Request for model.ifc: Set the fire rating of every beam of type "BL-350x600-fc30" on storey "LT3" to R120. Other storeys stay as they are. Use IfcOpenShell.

First a look at what the model holds.

```python
import ifcopenshell
import ifcopenshell.util.element

model = ifcopenshell.open("model.ifc")
print(model.schema)
storey = next(s for s in model.by_type("IfcBuildingStorey") if s.Name == "LT3")
beams = [e for e in ifcopenshell.util.element.get_decomposition(storey) if e.is_a("IfcBeam")]
seen = {}
for e in beams:
    element_type = ifcopenshell.util.element.get_type(e)
    key = (element_type.Name if element_type != e and element_type else None, ifcopenshell.util.element.get_pset(e, "Pset_BeamCommon", "FireRating"))
    seen[key] = seen.get(key, 0) + 1
for (name, value), count in sorted(seen.items(), key=str):
    print(count, "x", name, "|", value)
```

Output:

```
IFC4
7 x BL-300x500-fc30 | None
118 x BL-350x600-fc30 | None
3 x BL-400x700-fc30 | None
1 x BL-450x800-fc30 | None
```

```python
import ifcopenshell
import ifcopenshell.api.pset
import ifcopenshell.util.element

model = ifcopenshell.open("model.ifc")

storey = next(s for s in model.by_type("IfcBuildingStorey") if s.Name == "LT3")
beams = [e for e in ifcopenshell.util.element.get_decomposition(storey) if e.is_a("IfcBeam")]

count = 0
for e in beams:
    element_type = ifcopenshell.util.element.get_type(e)
    if element_type in (None, e) or element_type.Name != "BL-350x600-fc30":
        continue
    # add_pset returns the element's existing set when there is one.
    pset = ifcopenshell.api.pset.add_pset(model, product=e, name="Pset_BeamCommon")
    ifcopenshell.api.pset.edit_pset(model, pset=pset, properties={"FireRating": "R120"})
    count += 1

print(count, "beams updated")

model.write("model_edited.ifc")
```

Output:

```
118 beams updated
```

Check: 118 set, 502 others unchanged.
